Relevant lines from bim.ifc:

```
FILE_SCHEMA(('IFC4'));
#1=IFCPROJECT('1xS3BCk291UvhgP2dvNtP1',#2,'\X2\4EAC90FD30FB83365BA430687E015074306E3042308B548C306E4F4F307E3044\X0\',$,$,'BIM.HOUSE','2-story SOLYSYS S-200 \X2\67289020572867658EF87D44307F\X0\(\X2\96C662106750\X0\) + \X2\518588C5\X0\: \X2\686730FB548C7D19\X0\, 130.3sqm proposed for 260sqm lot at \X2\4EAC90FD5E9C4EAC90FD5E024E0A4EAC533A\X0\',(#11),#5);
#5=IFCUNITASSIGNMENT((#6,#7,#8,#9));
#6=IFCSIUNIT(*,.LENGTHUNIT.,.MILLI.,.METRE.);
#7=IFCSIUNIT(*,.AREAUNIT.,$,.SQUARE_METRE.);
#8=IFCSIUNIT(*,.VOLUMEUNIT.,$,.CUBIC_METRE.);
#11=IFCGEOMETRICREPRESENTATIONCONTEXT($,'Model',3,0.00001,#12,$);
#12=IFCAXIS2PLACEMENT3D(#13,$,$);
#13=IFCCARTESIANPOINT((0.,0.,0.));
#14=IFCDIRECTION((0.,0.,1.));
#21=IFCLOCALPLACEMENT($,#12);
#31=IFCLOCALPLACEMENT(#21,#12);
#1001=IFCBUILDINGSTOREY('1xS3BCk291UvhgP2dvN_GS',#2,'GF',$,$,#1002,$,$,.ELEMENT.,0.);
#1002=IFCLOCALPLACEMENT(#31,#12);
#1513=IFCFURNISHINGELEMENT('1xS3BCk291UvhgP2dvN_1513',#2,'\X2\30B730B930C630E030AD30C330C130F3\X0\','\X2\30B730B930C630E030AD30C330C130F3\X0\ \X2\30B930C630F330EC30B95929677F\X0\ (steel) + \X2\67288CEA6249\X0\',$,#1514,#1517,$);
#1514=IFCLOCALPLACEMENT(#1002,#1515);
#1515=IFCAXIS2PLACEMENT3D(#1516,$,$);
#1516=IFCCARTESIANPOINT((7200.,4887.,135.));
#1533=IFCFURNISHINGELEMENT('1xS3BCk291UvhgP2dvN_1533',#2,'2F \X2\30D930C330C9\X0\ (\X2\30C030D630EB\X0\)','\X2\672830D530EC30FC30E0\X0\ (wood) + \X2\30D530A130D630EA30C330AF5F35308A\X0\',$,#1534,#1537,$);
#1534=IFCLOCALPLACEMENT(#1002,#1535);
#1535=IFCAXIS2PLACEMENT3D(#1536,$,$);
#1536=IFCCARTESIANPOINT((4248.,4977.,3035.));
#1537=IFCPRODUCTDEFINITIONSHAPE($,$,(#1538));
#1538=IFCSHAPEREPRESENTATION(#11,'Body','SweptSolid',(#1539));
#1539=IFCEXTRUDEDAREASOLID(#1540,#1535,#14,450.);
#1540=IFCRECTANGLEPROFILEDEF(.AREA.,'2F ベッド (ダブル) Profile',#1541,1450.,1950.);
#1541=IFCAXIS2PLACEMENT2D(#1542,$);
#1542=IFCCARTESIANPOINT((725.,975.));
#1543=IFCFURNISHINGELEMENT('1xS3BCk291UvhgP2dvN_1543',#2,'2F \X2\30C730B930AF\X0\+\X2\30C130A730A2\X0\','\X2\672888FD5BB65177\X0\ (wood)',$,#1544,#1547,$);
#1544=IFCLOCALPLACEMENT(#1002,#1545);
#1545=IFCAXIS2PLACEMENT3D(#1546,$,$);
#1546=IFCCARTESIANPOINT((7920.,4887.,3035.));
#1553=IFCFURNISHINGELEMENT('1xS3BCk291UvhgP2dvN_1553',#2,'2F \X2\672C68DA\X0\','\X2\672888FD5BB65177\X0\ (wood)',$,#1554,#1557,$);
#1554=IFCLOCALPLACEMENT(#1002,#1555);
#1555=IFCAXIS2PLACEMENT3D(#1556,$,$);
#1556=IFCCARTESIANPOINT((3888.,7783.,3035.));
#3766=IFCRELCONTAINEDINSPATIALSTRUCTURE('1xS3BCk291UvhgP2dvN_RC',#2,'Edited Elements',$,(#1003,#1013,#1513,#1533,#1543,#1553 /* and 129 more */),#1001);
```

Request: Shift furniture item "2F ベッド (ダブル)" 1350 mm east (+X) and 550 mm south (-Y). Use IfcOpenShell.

```python
import ifcopenshell
import ifcopenshell.api.geometry
import ifcopenshell.util.placement

model = ifcopenshell.open("bim.ifc")

item = model.by_guid("1xS3BCk291UvhgP2dvN_1533")
matrix = ifcopenshell.util.placement.get_local_placement(item.ObjectPlacement)
matrix[0, 3] += 1350.0
matrix[1, 3] -= 550.0
ifcopenshell.api.geometry.edit_object_placement(model, product=item, matrix=matrix, is_si=False)

print(ifcopenshell.util.placement.get_local_placement(item.ObjectPlacement).round(3) + 0.0)

model.write("bim_edited.ifc")
```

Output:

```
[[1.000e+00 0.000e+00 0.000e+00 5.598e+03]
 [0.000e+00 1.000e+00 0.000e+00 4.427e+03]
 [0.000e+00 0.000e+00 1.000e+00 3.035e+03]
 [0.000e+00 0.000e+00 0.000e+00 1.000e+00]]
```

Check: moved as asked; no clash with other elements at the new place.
